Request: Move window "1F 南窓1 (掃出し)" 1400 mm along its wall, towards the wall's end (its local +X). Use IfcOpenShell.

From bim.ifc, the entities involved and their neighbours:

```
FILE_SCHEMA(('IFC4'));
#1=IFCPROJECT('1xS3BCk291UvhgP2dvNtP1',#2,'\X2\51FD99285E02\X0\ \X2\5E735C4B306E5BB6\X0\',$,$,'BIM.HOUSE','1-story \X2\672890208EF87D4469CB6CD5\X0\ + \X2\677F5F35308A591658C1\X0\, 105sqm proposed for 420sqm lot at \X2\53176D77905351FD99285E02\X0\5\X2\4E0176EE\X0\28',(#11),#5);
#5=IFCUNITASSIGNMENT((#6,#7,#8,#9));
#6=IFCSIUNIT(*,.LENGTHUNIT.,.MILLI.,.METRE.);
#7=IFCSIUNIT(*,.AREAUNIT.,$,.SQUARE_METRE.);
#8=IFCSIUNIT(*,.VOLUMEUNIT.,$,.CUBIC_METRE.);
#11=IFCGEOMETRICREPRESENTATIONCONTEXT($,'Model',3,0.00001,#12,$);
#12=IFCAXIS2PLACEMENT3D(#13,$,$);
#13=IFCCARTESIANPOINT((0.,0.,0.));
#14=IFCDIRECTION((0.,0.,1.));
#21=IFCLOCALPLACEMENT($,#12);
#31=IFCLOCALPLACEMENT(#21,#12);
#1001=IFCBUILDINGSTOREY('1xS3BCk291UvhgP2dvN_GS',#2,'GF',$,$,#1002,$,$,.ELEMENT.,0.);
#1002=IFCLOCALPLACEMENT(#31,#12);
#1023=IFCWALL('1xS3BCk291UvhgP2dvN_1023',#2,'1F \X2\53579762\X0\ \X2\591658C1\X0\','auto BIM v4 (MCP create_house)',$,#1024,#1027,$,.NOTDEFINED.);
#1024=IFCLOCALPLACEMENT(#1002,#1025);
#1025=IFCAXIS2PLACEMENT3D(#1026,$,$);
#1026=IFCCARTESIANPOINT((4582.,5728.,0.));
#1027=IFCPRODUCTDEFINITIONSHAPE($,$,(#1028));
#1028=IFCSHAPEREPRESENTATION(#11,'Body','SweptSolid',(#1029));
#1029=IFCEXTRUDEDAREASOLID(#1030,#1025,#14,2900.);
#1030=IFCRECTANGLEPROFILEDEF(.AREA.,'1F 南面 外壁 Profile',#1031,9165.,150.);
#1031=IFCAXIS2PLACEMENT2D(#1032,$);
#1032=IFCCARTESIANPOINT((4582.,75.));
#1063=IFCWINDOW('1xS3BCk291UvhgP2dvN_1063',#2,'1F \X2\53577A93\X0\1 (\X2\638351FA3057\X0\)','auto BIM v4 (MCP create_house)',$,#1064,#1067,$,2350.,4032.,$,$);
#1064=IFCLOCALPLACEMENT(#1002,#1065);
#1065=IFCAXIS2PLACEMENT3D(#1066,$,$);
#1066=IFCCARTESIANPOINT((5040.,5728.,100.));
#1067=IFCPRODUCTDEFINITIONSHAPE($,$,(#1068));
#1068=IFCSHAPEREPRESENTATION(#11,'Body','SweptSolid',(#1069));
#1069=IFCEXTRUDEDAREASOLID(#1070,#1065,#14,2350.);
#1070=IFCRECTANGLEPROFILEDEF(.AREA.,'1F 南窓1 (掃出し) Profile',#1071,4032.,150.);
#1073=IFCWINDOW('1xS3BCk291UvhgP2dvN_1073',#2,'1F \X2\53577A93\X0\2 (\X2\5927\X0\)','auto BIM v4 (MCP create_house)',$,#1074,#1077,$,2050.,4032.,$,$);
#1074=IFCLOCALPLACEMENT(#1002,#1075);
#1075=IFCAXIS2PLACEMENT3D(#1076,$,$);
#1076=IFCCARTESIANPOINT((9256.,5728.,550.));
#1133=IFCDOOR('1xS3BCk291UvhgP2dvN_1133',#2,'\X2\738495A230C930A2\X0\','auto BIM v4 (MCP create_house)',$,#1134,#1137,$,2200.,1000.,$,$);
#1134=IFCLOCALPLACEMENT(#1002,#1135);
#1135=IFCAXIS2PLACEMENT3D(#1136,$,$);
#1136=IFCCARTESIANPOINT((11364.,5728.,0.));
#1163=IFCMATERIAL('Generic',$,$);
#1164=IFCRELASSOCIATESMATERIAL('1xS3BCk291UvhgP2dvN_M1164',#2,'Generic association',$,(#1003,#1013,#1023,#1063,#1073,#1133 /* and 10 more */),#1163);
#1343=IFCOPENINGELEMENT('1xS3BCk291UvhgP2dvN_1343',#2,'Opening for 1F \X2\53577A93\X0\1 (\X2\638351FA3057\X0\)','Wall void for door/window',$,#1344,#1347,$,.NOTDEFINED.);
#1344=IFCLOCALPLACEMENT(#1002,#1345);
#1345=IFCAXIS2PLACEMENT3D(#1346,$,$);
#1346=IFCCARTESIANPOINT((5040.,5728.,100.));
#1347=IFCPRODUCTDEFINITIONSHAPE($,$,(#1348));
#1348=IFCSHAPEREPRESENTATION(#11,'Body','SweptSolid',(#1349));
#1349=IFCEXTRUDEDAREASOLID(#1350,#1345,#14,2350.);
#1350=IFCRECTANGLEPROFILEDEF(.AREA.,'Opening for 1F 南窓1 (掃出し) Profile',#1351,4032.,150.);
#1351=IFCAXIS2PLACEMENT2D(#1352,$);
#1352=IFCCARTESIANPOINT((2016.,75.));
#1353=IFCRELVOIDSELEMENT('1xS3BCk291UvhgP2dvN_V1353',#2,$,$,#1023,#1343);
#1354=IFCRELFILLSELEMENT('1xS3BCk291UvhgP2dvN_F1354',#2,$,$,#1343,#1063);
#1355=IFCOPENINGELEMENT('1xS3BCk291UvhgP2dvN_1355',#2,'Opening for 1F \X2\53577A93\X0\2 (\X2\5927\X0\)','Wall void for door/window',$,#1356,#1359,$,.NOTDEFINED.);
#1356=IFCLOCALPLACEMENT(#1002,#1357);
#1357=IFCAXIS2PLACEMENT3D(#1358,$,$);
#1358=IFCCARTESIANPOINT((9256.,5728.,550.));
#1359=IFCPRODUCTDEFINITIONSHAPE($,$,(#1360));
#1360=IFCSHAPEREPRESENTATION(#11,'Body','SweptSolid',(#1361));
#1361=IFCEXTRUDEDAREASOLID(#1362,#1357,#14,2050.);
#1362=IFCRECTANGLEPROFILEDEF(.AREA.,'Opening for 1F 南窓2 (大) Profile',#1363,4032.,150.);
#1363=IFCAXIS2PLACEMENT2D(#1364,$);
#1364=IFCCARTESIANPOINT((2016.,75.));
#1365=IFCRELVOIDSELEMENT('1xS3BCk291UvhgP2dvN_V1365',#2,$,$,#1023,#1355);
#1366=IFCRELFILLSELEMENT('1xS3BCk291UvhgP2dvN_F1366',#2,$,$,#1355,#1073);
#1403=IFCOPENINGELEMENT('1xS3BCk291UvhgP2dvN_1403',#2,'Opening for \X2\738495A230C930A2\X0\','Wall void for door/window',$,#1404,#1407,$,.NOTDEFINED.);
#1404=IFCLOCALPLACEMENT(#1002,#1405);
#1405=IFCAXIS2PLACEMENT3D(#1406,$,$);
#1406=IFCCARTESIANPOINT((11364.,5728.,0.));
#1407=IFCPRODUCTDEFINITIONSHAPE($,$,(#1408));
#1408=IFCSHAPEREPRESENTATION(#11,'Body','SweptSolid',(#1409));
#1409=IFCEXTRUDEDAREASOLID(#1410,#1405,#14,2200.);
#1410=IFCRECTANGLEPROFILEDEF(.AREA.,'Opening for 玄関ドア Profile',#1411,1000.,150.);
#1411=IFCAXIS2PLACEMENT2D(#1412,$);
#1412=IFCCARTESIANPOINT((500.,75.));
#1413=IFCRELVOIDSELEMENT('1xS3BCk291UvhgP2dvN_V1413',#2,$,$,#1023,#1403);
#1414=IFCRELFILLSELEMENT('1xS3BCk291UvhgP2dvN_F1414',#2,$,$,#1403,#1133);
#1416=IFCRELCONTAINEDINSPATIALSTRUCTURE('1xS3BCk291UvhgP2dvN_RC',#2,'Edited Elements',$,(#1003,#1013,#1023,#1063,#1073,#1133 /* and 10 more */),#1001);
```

```python
import ifcopenshell
import ifcopenshell.api.geometry
import ifcopenshell.util.placement
import ifcopenshell.util.unit

model = ifcopenshell.open("bim.ifc")
unit_scale = ifcopenshell.util.unit.calculate_unit_scale(model)

window = model.by_guid("1xS3BCk291UvhgP2dvN_1063")
opening = window.FillsVoids[0].RelatingOpeningElement
wall = opening.VoidsElements[0].RelatingBuildingElement

wall_matrix = ifcopenshell.util.placement.get_local_placement(wall.ObjectPlacement)
shift = wall_matrix[:3, 0] * 1.4 / unit_scale
before = ifcopenshell.util.placement.get_local_placement(window.ObjectPlacement)[:3, 3].copy()

# The window is not placed relative to its opening, so move both.
for product in (opening, window):
    matrix = ifcopenshell.util.placement.get_local_placement(product.ObjectPlacement)
    matrix[:3, 3] += shift
    ifcopenshell.api.geometry.edit_object_placement(model, product=product, matrix=matrix, is_si=False)

after = ifcopenshell.util.placement.get_local_placement(window.ObjectPlacement)[:3, 3]
print("window moved by", (after - before).round(3) + 0.0)

model.write("bim_updated.ifc")
```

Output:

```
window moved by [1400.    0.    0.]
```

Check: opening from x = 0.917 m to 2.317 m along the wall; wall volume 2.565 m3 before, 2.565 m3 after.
